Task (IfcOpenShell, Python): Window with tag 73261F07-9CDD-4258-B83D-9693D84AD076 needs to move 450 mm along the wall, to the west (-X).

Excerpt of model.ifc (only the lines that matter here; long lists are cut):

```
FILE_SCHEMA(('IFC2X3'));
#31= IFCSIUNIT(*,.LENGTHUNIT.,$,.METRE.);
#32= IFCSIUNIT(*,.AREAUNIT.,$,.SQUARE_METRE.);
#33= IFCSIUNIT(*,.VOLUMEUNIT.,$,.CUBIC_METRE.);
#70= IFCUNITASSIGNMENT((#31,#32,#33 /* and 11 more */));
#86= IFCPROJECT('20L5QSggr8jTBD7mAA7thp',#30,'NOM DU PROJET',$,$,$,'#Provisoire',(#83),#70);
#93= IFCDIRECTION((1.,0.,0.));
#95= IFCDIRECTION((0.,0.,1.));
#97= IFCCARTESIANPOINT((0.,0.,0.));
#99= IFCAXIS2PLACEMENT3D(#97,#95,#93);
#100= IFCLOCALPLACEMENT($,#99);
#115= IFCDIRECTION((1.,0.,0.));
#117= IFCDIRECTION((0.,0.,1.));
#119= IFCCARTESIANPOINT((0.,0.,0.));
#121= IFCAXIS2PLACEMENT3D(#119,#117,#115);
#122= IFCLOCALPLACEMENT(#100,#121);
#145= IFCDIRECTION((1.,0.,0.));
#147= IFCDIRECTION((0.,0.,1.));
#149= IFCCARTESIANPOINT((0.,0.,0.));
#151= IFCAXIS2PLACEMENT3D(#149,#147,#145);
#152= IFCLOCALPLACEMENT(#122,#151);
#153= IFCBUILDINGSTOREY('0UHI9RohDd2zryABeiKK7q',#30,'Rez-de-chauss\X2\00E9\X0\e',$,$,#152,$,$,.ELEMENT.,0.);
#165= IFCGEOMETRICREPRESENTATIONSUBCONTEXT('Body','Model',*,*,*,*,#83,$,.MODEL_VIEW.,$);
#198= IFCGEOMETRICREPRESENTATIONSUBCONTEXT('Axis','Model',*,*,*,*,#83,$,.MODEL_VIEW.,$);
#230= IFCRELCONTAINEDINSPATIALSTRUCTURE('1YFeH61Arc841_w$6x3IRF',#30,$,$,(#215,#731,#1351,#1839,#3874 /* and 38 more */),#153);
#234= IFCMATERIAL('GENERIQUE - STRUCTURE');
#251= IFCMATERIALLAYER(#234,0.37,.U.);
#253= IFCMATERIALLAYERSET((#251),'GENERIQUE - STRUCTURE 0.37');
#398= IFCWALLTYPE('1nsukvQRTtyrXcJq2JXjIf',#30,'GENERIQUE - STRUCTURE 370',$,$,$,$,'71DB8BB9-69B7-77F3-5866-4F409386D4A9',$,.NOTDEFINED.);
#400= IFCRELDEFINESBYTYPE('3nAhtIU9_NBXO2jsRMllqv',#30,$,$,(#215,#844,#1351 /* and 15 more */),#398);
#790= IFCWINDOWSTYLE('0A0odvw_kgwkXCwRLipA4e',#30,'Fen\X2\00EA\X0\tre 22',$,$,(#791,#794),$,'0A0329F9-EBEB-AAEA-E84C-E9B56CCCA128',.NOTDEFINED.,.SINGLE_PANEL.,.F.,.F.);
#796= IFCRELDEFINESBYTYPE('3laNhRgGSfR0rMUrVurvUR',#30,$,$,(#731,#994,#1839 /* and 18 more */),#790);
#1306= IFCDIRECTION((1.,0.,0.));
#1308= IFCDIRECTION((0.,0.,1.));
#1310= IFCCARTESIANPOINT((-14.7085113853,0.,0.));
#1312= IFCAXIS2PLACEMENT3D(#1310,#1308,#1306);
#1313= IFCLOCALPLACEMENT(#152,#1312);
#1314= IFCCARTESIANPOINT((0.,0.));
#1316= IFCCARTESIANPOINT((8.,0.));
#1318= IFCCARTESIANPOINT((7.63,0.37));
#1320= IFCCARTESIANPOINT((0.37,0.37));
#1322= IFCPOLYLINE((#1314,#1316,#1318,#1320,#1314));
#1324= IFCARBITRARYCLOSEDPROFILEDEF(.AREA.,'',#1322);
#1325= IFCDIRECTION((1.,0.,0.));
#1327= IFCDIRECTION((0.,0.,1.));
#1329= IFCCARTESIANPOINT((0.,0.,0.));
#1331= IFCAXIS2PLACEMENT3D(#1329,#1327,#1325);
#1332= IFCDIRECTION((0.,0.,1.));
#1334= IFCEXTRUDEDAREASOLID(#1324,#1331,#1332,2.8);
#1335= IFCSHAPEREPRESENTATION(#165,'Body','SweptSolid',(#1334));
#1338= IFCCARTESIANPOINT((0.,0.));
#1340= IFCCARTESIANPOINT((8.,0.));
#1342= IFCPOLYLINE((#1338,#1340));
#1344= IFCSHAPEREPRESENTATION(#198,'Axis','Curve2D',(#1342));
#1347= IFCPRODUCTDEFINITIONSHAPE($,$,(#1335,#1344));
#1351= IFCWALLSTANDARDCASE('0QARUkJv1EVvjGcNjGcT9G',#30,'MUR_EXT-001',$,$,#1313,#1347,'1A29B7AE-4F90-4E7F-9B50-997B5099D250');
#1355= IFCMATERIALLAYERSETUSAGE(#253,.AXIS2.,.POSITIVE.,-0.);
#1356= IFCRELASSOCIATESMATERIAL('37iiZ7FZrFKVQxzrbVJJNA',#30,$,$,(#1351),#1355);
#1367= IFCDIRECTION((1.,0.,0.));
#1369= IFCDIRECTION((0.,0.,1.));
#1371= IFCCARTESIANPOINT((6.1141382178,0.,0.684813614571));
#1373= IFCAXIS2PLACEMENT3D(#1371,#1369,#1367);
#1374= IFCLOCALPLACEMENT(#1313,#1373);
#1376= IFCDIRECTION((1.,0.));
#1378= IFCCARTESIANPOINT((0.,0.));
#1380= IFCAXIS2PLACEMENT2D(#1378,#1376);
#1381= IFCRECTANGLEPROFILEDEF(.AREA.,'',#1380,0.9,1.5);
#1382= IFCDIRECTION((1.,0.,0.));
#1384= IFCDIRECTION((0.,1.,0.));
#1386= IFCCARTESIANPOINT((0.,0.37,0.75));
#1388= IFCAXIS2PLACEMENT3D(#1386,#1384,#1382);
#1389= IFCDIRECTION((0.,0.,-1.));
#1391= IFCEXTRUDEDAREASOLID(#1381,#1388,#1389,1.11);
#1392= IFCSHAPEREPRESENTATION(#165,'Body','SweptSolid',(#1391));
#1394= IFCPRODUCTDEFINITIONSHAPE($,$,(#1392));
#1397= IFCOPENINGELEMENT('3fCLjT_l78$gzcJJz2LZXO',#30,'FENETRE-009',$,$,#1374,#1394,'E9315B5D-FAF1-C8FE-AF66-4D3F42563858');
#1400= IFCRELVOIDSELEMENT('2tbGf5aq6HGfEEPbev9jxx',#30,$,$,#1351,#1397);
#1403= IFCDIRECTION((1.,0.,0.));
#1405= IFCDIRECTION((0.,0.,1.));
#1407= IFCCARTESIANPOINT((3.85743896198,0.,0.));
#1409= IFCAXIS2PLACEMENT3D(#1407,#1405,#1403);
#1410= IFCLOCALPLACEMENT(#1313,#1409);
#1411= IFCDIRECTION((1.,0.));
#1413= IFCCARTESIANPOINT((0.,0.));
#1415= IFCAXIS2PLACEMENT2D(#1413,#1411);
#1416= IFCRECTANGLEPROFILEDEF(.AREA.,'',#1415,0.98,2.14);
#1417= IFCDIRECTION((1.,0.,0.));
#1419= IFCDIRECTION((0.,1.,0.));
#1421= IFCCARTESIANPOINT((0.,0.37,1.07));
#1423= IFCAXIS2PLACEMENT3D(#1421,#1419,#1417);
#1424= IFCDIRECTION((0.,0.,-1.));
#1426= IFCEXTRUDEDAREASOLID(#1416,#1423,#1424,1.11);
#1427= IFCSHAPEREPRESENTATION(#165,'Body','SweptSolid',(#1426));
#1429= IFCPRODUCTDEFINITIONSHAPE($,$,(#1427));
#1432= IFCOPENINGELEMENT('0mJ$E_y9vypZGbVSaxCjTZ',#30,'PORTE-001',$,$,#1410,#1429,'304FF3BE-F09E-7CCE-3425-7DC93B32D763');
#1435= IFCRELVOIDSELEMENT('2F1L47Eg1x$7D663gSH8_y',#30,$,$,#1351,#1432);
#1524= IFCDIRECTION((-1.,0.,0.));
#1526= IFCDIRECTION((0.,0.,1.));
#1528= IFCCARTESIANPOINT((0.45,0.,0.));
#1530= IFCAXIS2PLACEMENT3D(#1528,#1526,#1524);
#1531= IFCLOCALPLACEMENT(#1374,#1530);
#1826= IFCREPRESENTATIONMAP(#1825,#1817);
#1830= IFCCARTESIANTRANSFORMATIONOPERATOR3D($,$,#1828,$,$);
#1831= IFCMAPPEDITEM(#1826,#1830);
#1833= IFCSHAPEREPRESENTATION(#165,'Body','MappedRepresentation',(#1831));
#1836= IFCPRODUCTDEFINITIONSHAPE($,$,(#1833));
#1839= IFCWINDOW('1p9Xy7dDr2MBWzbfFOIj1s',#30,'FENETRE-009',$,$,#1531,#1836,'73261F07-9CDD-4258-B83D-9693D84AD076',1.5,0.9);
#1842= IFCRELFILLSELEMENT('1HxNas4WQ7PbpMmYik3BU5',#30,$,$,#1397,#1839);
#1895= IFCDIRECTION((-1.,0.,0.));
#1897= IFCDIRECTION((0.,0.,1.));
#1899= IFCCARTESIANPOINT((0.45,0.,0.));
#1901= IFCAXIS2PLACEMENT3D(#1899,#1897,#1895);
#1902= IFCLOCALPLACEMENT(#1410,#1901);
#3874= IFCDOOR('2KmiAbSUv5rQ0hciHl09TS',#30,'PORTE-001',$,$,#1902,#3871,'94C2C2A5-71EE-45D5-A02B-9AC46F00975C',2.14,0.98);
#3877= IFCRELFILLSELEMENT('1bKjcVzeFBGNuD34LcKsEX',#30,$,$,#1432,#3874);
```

```python
import ifcopenshell
import ifcopenshell.api.geometry
import ifcopenshell.util.placement
import ifcopenshell.util.unit

model = ifcopenshell.open("model.ifc")
unit_scale = ifcopenshell.util.unit.calculate_unit_scale(model)

window = model.by_guid("1p9Xy7dDr2MBWzbfFOIj1s")
opening = window.FillsVoids[0].RelatingOpeningElement
wall = opening.VoidsElements[0].RelatingBuildingElement

wall_matrix = ifcopenshell.util.placement.get_local_placement(wall.ObjectPlacement)
shift = wall_matrix[:3, 0] * -0.45 / unit_scale
before = ifcopenshell.util.placement.get_local_placement(window.ObjectPlacement)[:3, 3].copy()

# The window is placed relative to its opening, so it follows when the opening moves.
matrix = ifcopenshell.util.placement.get_local_placement(opening.ObjectPlacement)
matrix[:3, 3] += shift
ifcopenshell.api.geometry.edit_object_placement(
    model, product=opening, matrix=matrix, is_si=False, should_transform_children=True
)

after = ifcopenshell.util.placement.get_local_placement(window.ObjectPlacement)[:3, 3]
print("window moved by", (after - before).round(3) + 0.0)

model.write("model_edited.ifc")
```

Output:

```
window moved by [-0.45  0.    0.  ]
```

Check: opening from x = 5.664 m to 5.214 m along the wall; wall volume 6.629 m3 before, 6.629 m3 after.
